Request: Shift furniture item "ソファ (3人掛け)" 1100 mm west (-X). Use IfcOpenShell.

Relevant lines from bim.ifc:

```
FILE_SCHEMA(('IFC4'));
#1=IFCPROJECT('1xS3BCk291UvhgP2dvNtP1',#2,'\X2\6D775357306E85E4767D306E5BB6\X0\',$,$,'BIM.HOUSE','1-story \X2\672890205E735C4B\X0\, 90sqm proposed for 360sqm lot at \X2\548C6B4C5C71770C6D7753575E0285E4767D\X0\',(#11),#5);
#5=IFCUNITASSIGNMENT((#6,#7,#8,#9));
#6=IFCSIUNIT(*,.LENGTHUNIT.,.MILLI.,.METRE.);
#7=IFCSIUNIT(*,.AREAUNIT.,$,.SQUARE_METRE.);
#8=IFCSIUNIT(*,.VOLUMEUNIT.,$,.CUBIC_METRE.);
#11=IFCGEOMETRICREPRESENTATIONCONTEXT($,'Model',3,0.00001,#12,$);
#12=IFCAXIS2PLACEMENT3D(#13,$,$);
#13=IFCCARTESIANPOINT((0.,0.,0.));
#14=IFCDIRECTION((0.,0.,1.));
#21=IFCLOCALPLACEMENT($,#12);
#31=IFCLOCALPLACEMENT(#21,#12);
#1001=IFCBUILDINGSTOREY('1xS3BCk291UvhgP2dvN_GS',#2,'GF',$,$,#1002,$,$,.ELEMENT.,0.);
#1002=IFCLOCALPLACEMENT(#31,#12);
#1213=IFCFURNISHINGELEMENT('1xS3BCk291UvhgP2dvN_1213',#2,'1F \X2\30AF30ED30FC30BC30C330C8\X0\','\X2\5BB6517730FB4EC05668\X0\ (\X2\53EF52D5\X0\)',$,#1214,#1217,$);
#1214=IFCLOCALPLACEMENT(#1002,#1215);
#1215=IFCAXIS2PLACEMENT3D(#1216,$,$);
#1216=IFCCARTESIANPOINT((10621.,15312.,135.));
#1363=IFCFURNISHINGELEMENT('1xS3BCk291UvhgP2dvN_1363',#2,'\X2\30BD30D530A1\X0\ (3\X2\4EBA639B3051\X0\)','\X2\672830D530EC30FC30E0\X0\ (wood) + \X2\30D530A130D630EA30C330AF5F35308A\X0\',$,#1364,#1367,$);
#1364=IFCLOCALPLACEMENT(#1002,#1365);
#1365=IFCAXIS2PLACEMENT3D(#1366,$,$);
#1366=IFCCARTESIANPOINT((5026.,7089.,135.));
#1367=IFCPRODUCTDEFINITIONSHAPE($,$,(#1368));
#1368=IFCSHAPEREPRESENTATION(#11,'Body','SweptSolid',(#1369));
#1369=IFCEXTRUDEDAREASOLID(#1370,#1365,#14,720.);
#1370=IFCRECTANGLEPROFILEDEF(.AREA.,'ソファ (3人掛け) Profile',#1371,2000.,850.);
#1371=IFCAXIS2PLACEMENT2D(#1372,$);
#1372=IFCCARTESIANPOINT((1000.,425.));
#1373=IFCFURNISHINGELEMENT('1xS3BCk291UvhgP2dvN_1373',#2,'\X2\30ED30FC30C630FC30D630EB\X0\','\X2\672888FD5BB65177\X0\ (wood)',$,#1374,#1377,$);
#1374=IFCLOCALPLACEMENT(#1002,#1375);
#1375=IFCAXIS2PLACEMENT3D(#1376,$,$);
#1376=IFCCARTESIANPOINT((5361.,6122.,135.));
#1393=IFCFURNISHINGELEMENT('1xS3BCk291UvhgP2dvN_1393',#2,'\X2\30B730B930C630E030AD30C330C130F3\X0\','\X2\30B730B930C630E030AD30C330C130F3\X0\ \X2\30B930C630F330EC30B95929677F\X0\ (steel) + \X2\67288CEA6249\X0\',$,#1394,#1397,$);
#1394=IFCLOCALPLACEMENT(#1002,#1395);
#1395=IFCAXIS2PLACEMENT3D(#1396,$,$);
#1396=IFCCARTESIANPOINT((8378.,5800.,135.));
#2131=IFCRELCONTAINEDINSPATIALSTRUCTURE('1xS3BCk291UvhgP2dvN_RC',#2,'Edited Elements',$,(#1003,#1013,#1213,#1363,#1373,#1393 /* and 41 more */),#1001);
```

```python
import ifcopenshell
import ifcopenshell.api.geometry
import ifcopenshell.util.placement
import ifcopenshell.util.unit

model = ifcopenshell.open("bim.ifc")
unit_scale = ifcopenshell.util.unit.calculate_unit_scale(model)

item = model.by_guid("1xS3BCk291UvhgP2dvN_1363")
matrix = ifcopenshell.util.placement.get_local_placement(item.ObjectPlacement)
matrix[0, 3] -= 1.1 / unit_scale
ifcopenshell.api.geometry.edit_object_placement(model, product=item, matrix=matrix, is_si=False)

print(ifcopenshell.util.placement.get_local_placement(item.ObjectPlacement).round(3) + 0.0)

model.write("bim_v2.ifc")
```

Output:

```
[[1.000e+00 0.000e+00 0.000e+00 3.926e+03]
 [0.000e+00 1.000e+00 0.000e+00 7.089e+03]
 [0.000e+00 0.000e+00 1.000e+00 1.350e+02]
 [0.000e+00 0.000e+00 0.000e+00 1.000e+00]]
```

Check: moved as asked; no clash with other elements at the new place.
